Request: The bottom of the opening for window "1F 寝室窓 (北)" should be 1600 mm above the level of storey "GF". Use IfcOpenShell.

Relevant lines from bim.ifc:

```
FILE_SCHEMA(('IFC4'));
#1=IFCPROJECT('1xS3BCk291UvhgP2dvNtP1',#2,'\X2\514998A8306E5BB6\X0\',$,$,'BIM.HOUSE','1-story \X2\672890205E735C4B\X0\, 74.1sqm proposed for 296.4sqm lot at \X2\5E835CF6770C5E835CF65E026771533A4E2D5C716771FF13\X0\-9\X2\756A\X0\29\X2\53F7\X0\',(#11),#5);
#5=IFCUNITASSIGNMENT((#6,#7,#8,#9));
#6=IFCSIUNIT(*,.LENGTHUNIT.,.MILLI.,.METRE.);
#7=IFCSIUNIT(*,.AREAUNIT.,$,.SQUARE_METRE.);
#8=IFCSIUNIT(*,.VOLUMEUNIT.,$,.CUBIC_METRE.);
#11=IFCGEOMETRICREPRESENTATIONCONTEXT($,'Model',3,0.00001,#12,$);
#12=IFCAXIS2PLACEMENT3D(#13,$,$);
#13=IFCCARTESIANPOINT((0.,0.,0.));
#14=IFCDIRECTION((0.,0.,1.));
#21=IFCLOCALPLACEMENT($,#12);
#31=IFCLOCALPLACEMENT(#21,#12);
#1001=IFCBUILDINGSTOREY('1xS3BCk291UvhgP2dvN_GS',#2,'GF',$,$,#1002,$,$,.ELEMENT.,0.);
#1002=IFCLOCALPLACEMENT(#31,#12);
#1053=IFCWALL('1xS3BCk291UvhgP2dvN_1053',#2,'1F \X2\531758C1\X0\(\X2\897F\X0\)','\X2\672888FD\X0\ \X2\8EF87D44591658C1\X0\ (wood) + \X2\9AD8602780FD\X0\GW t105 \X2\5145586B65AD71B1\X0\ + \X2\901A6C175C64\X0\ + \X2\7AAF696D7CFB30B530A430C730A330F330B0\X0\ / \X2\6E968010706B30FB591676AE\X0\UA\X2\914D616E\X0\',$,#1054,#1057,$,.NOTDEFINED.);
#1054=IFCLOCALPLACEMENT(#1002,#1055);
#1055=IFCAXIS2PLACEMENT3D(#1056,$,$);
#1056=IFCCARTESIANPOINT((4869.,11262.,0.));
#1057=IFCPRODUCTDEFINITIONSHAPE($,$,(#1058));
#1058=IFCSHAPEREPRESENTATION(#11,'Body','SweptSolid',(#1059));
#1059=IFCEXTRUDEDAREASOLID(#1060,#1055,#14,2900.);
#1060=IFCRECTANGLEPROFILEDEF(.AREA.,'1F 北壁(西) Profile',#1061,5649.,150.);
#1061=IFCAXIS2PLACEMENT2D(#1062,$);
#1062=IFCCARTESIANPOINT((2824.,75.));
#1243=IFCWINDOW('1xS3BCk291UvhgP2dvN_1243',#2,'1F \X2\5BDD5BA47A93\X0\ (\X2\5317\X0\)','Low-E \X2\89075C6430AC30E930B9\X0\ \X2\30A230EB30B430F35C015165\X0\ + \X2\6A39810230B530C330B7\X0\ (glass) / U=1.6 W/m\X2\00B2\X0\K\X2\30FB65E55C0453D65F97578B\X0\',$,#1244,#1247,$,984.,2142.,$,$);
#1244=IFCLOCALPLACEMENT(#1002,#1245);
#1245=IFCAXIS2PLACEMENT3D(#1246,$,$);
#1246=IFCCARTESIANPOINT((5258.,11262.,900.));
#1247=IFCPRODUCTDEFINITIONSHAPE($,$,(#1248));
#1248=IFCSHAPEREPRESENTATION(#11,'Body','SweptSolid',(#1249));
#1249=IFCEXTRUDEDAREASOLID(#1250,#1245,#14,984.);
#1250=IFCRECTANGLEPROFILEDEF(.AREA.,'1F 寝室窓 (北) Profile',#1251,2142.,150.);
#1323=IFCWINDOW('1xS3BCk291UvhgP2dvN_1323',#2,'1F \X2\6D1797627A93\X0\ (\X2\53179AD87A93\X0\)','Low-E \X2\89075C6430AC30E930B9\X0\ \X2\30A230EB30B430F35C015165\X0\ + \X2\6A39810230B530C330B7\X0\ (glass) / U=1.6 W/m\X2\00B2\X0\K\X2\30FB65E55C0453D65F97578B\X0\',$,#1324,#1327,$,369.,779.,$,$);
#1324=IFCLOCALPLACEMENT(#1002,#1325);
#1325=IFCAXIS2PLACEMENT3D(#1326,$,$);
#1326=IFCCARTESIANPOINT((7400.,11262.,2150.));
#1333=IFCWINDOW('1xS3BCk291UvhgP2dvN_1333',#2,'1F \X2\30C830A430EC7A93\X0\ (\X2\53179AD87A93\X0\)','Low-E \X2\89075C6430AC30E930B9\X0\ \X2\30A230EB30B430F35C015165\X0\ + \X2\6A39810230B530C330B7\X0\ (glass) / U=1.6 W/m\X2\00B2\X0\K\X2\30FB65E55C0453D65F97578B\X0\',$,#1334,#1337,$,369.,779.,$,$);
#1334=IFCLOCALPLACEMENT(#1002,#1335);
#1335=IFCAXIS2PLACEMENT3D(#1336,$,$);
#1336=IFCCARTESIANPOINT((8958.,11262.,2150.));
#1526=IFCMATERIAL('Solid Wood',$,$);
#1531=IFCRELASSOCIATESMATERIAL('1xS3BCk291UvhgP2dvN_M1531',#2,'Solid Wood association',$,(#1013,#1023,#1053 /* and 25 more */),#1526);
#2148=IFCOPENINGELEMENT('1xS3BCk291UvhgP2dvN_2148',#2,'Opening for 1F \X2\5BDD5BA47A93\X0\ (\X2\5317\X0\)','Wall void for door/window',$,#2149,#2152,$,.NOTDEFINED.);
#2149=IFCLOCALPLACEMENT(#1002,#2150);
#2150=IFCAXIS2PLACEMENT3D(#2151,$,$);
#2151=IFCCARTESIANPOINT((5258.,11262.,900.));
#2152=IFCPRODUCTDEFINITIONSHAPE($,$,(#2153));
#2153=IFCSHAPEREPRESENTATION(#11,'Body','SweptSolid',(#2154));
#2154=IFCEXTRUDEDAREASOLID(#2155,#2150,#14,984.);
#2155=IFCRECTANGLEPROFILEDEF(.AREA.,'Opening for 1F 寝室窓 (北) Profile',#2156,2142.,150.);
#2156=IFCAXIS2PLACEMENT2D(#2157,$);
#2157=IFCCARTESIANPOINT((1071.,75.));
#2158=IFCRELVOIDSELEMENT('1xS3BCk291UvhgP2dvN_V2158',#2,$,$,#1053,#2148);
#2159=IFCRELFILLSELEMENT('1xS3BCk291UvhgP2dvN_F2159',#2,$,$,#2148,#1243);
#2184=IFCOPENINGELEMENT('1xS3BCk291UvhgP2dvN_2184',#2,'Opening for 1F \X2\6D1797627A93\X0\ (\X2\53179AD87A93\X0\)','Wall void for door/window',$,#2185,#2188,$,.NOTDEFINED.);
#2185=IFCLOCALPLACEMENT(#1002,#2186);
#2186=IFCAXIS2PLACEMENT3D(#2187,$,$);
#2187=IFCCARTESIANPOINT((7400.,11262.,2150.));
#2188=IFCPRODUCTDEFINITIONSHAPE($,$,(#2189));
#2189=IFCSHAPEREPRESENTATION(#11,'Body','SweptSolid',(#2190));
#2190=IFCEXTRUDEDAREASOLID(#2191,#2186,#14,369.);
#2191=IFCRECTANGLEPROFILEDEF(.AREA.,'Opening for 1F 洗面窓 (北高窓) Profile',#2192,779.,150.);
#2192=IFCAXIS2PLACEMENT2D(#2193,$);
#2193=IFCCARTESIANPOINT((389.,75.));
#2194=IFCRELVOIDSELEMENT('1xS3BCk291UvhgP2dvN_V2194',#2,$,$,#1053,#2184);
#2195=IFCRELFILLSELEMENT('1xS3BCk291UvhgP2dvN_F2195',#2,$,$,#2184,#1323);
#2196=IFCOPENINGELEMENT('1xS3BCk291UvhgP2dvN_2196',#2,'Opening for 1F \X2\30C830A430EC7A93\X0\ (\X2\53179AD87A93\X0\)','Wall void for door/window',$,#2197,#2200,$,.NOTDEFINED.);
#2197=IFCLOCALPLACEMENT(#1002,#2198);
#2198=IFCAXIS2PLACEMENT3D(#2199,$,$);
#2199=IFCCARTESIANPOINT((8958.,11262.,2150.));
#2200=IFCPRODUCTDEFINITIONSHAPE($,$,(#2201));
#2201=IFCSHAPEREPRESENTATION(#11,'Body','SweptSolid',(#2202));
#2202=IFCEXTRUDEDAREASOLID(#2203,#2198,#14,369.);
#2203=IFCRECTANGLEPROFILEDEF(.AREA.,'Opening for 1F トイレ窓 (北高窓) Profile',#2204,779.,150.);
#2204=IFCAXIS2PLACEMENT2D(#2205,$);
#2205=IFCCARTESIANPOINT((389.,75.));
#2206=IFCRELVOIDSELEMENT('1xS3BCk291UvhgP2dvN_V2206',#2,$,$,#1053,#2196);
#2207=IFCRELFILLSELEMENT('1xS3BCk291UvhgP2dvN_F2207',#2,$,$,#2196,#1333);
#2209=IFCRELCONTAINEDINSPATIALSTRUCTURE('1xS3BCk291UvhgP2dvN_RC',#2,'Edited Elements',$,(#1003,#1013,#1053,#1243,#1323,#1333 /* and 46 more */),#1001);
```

```python
import numpy as np
import ifcopenshell
import ifcopenshell.api.geometry
import ifcopenshell.geom
import ifcopenshell.util.element
import ifcopenshell.util.placement
import ifcopenshell.util.shape
import ifcopenshell.util.unit

model = ifcopenshell.open("bim.ifc")
unit_scale = ifcopenshell.util.unit.calculate_unit_scale(model)

window = model.by_guid("1xS3BCk291UvhgP2dvN_1243")
opening = window.FillsVoids[0].RelatingOpeningElement
storey = ifcopenshell.util.element.get_container(window, ifc_class="IfcBuildingStorey")
level = ifcopenshell.util.placement.get_local_placement(storey.ObjectPlacement)[2, 3]

# The opening's origin need not be at the sill, so measure its lowest point.
shape = ifcopenshell.geom.create_shape(ifcopenshell.geom.settings(), opening)
bottom = ifcopenshell.util.shape.get_shape_bottom_elevation(shape, shape.geometry) / unit_scale
dz = level + 1.6 / unit_scale - bottom

shift = np.array([0.0, 0.0, dz])
# The window is not placed relative to its opening, so move both.
for product in (opening, window):
    matrix = ifcopenshell.util.placement.get_local_placement(product.ObjectPlacement)
    matrix[:3, 3] += shift
    ifcopenshell.api.geometry.edit_object_placement(model, product=product, matrix=matrix, is_si=False)

print(f"moved by {dz * unit_scale:+.3f} m")

model.write("bim_v2.ifc")
```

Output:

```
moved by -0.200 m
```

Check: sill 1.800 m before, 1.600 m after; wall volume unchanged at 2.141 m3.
